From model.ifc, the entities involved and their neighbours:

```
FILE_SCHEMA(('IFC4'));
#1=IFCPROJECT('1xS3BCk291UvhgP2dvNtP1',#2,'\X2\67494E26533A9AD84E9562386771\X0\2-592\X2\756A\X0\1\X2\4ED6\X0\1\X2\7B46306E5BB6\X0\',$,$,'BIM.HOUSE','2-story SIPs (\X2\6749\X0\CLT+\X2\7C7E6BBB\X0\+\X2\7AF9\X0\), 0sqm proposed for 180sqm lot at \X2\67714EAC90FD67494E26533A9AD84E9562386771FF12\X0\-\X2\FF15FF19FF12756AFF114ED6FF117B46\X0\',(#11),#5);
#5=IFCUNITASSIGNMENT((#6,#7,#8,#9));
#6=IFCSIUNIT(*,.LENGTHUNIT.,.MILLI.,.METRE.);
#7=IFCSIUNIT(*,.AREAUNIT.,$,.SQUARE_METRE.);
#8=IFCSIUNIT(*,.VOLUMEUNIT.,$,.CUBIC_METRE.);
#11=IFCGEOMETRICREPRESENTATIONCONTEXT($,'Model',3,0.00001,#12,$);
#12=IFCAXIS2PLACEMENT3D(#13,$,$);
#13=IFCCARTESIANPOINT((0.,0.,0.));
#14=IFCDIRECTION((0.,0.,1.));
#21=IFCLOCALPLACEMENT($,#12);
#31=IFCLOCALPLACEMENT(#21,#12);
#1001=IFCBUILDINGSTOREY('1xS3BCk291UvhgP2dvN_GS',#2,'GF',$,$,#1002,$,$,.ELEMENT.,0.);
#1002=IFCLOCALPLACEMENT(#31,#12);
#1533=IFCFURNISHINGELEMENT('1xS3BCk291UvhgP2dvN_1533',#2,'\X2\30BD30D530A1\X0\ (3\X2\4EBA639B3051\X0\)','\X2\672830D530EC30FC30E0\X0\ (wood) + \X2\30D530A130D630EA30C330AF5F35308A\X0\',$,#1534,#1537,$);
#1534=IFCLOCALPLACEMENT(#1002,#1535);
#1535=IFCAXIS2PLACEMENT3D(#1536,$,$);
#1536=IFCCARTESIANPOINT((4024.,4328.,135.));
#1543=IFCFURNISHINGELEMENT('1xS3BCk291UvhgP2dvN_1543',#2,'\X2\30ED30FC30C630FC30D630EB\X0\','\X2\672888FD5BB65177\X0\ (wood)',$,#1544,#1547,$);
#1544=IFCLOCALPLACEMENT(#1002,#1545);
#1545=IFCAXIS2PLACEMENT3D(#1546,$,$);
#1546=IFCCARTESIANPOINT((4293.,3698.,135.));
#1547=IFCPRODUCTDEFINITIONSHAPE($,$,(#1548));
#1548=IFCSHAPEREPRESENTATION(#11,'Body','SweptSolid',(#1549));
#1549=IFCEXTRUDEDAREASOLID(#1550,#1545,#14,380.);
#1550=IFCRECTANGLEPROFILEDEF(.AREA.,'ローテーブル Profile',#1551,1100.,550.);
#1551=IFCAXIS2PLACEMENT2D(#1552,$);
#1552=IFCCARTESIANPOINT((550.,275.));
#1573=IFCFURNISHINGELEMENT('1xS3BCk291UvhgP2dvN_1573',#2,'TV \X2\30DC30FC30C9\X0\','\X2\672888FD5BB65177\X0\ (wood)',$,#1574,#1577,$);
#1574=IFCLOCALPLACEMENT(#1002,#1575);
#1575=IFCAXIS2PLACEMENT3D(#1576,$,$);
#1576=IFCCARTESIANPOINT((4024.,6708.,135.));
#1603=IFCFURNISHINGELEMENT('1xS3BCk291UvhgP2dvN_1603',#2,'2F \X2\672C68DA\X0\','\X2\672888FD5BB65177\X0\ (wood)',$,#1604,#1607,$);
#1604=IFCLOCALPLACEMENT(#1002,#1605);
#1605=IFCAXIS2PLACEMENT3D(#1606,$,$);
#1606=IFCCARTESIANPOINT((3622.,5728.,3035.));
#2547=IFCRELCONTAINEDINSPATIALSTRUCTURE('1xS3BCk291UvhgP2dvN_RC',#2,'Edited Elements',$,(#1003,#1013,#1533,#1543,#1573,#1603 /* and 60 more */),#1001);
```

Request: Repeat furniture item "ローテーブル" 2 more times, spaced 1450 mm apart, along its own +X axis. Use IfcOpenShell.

```python
import ifcopenshell
import ifcopenshell.api.geometry
import ifcopenshell.api.root
import ifcopenshell.util.element
import ifcopenshell.util.placement

model = ifcopenshell.open("model.ifc")


def reuse_history(source, copy):
    """copy_class also copies each property set's owner history, people and application; keep the originals."""
    for rel in copy.IsDefinedBy:
        if rel.is_a("IfcRelDefinesByProperties") and (history := rel.RelatingPropertyDefinition.OwnerHistory):
            rel.RelatingPropertyDefinition.OwnerHistory = source.OwnerHistory
            ifcopenshell.util.element.remove_deep2(model, history)


source = model.by_guid("1xS3BCk291UvhgP2dvN_1543")
base = ifcopenshell.util.placement.get_local_placement(source.ObjectPlacement)
step = base[:3, 0] * 1450.0

for i in range(1, 3):
    copy = ifcopenshell.api.root.copy_class(model, product=source)
    copy.Representation = ifcopenshell.util.element.copy_deep(
        model, source.Representation, exclude=["IfcGeometricRepresentationContext", "IfcRepresentationMap"]
    )
    reuse_history(source, copy)
    matrix = base.copy()
    matrix[:3, 3] += i * step
    print("added at", matrix[:3, 3].round(3) + 0.0)
    ifcopenshell.api.geometry.edit_object_placement(model, product=copy, matrix=matrix, is_si=False)

model.write("model_rev.ifc")
```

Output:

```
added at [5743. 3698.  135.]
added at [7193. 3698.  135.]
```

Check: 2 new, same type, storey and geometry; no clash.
